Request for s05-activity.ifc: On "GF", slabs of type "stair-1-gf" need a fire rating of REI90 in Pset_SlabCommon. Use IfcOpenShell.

First a look at what the model holds.

```python
import ifcopenshell
import ifcopenshell.util.element

model = ifcopenshell.open("s05-activity.ifc")
print(model.schema)
storey = next(s for s in model.by_type("IfcBuildingStorey") if s.Name == "GF")
slabs = [e for e in ifcopenshell.util.element.get_decomposition(storey) if e.is_a("IfcSlab")]
seen = {}
for e in slabs:
    element_type = ifcopenshell.util.element.get_type(e)
    key = (element_type.Name if element_type != e and element_type else None, ifcopenshell.util.element.get_pset(e, "Pset_SlabCommon", "FireRating"))
    seen[key] = seen.get(key, 0) + 1
for (name, value), count in sorted(seen.items(), key=str):
    print(count, "x", name, "|", value)
```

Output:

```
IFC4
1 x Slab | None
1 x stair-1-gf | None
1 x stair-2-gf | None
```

```python
import ifcopenshell
import ifcopenshell.api.pset
import ifcopenshell.util.element

model = ifcopenshell.open("s05-activity.ifc")

storey = next(s for s in model.by_type("IfcBuildingStorey") if s.Name == "GF")
slabs = [e for e in ifcopenshell.util.element.get_decomposition(storey) if e.is_a("IfcSlab")]

count = 0
for e in slabs:
    element_type = ifcopenshell.util.element.get_type(e)
    if element_type in (None, e) or element_type.Name != "stair-1-gf":
        continue
    # add_pset returns the element's existing set when there is one.
    pset = ifcopenshell.api.pset.add_pset(model, product=e, name="Pset_SlabCommon")
    ifcopenshell.api.pset.edit_pset(model, pset=pset, properties={"FireRating": "REI90"})
    count += 1

print(count, "slabs updated")

model.write("s05-activity_edited.ifc")
```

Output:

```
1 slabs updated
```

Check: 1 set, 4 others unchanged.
